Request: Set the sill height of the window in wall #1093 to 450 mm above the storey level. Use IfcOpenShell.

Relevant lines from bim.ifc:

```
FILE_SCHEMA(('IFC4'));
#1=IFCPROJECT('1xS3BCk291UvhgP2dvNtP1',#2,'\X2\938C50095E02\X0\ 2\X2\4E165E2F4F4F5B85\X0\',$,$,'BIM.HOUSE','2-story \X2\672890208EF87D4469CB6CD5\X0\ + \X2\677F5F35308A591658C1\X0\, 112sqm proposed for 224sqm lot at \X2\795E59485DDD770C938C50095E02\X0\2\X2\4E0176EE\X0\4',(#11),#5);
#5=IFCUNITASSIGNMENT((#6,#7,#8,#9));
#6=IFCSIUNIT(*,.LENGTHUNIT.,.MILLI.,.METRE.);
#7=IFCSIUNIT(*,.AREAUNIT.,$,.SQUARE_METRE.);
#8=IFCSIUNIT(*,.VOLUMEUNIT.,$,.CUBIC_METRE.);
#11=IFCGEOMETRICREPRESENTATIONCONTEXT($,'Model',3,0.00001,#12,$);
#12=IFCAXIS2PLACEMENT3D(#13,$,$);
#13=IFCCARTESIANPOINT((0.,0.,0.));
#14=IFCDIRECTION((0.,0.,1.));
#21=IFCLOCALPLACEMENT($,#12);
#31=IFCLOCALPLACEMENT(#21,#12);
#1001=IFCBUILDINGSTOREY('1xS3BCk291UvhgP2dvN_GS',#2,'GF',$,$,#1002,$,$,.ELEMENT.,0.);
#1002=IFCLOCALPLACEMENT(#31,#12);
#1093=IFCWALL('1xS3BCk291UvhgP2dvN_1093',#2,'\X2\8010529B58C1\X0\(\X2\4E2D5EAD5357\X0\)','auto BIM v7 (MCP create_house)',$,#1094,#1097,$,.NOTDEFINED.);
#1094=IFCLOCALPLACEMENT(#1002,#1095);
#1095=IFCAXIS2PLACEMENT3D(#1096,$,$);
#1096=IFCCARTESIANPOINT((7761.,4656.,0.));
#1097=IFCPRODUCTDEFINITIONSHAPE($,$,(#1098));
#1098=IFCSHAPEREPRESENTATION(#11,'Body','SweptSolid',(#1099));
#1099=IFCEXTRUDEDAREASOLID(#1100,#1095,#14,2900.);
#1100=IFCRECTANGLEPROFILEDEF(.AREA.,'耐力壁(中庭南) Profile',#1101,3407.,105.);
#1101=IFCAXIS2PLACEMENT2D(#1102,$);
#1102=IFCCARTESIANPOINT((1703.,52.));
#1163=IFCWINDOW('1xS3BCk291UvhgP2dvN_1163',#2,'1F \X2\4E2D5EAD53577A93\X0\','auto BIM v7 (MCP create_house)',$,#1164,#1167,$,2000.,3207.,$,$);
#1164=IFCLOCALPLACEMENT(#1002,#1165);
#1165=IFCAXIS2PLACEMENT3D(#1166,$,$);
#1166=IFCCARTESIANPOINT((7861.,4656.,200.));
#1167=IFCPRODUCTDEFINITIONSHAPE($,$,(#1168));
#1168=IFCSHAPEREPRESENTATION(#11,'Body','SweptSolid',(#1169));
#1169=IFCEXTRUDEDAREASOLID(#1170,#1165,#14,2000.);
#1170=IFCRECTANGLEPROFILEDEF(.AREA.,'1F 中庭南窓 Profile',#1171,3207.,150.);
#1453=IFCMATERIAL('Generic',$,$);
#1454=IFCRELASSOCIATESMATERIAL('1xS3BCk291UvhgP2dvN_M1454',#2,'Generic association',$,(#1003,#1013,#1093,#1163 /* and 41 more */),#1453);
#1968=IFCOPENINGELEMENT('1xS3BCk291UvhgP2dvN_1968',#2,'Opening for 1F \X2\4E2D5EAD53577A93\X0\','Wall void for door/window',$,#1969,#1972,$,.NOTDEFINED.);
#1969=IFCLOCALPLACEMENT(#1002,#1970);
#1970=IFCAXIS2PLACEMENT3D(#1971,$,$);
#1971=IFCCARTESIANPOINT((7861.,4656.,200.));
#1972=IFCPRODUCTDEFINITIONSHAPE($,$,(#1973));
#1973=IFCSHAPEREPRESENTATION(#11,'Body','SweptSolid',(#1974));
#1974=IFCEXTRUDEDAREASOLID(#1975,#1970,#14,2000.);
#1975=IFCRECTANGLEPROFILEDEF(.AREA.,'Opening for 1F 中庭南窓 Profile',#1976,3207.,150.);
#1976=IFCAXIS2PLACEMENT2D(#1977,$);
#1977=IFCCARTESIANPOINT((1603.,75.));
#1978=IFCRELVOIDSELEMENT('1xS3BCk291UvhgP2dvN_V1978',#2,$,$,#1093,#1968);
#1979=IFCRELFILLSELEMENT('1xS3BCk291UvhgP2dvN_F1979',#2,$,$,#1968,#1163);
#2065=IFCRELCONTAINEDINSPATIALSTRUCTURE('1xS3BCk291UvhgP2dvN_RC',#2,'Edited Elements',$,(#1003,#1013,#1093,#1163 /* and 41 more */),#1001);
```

```python
import numpy as np
import ifcopenshell
import ifcopenshell.api.geometry
import ifcopenshell.geom
import ifcopenshell.util.element
import ifcopenshell.util.placement
import ifcopenshell.util.shape
import ifcopenshell.util.unit

model = ifcopenshell.open("bim.ifc")
unit_scale = ifcopenshell.util.unit.calculate_unit_scale(model)

window = model.by_id(1163)
opening = window.FillsVoids[0].RelatingOpeningElement
storey = ifcopenshell.util.element.get_container(window, ifc_class="IfcBuildingStorey")
level = ifcopenshell.util.placement.get_local_placement(storey.ObjectPlacement)[2, 3]

# The opening's origin need not be at the sill, so measure its lowest point.
shape = ifcopenshell.geom.create_shape(ifcopenshell.geom.settings(), opening)
bottom = ifcopenshell.util.shape.get_shape_bottom_elevation(shape, shape.geometry) / unit_scale
dz = level + 0.45 / unit_scale - bottom

shift = np.array([0.0, 0.0, dz])
# The window is not placed relative to its opening, so move both.
for product in (opening, window):
    matrix = ifcopenshell.util.placement.get_local_placement(product.ObjectPlacement)
    matrix[:3, 3] += shift
    ifcopenshell.api.geometry.edit_object_placement(model, product=product, matrix=matrix, is_si=False)

print(f"moved by {dz * unit_scale:+.3f} m")

model.write("bim_v2.ifc")
```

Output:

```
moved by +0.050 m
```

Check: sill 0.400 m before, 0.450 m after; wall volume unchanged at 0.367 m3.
